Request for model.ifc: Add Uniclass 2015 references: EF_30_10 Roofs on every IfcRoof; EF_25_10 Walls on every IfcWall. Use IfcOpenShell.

First a look at what the model holds.

```python
import ifcopenshell

model = ifcopenshell.open("model.ifc")
print(model.schema)
print("classifications:", [c.Name for c in model.by_type("IfcClassification")])
for ifc_class in ("IfcDoor", "IfcRoof", "IfcStair", "IfcWall", "IfcWindow"):
    print(ifc_class, len(model.by_type(ifc_class)))
```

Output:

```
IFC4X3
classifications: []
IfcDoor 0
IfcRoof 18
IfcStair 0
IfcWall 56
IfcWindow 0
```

```python
import ifcopenshell
import ifcopenshell.api.classification

model = ifcopenshell.open("model.ifc")

system = ifcopenshell.api.classification.add_classification(model, classification="Uniclass 2015")

codes = {
    "IfcRoof": ("EF_30_10", "Roofs"),
    "IfcWall": ("EF_25_10", "Walls"),
}
for ifc_class, (code, name) in codes.items():
    products = model.by_type(ifc_class)
    ifcopenshell.api.classification.add_reference(
        model, products=products, classification=system, identification=code, name=name
    )
    print(code, len(products))

model.write("model_v2.ifc")
```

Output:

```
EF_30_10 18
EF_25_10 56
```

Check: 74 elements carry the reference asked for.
